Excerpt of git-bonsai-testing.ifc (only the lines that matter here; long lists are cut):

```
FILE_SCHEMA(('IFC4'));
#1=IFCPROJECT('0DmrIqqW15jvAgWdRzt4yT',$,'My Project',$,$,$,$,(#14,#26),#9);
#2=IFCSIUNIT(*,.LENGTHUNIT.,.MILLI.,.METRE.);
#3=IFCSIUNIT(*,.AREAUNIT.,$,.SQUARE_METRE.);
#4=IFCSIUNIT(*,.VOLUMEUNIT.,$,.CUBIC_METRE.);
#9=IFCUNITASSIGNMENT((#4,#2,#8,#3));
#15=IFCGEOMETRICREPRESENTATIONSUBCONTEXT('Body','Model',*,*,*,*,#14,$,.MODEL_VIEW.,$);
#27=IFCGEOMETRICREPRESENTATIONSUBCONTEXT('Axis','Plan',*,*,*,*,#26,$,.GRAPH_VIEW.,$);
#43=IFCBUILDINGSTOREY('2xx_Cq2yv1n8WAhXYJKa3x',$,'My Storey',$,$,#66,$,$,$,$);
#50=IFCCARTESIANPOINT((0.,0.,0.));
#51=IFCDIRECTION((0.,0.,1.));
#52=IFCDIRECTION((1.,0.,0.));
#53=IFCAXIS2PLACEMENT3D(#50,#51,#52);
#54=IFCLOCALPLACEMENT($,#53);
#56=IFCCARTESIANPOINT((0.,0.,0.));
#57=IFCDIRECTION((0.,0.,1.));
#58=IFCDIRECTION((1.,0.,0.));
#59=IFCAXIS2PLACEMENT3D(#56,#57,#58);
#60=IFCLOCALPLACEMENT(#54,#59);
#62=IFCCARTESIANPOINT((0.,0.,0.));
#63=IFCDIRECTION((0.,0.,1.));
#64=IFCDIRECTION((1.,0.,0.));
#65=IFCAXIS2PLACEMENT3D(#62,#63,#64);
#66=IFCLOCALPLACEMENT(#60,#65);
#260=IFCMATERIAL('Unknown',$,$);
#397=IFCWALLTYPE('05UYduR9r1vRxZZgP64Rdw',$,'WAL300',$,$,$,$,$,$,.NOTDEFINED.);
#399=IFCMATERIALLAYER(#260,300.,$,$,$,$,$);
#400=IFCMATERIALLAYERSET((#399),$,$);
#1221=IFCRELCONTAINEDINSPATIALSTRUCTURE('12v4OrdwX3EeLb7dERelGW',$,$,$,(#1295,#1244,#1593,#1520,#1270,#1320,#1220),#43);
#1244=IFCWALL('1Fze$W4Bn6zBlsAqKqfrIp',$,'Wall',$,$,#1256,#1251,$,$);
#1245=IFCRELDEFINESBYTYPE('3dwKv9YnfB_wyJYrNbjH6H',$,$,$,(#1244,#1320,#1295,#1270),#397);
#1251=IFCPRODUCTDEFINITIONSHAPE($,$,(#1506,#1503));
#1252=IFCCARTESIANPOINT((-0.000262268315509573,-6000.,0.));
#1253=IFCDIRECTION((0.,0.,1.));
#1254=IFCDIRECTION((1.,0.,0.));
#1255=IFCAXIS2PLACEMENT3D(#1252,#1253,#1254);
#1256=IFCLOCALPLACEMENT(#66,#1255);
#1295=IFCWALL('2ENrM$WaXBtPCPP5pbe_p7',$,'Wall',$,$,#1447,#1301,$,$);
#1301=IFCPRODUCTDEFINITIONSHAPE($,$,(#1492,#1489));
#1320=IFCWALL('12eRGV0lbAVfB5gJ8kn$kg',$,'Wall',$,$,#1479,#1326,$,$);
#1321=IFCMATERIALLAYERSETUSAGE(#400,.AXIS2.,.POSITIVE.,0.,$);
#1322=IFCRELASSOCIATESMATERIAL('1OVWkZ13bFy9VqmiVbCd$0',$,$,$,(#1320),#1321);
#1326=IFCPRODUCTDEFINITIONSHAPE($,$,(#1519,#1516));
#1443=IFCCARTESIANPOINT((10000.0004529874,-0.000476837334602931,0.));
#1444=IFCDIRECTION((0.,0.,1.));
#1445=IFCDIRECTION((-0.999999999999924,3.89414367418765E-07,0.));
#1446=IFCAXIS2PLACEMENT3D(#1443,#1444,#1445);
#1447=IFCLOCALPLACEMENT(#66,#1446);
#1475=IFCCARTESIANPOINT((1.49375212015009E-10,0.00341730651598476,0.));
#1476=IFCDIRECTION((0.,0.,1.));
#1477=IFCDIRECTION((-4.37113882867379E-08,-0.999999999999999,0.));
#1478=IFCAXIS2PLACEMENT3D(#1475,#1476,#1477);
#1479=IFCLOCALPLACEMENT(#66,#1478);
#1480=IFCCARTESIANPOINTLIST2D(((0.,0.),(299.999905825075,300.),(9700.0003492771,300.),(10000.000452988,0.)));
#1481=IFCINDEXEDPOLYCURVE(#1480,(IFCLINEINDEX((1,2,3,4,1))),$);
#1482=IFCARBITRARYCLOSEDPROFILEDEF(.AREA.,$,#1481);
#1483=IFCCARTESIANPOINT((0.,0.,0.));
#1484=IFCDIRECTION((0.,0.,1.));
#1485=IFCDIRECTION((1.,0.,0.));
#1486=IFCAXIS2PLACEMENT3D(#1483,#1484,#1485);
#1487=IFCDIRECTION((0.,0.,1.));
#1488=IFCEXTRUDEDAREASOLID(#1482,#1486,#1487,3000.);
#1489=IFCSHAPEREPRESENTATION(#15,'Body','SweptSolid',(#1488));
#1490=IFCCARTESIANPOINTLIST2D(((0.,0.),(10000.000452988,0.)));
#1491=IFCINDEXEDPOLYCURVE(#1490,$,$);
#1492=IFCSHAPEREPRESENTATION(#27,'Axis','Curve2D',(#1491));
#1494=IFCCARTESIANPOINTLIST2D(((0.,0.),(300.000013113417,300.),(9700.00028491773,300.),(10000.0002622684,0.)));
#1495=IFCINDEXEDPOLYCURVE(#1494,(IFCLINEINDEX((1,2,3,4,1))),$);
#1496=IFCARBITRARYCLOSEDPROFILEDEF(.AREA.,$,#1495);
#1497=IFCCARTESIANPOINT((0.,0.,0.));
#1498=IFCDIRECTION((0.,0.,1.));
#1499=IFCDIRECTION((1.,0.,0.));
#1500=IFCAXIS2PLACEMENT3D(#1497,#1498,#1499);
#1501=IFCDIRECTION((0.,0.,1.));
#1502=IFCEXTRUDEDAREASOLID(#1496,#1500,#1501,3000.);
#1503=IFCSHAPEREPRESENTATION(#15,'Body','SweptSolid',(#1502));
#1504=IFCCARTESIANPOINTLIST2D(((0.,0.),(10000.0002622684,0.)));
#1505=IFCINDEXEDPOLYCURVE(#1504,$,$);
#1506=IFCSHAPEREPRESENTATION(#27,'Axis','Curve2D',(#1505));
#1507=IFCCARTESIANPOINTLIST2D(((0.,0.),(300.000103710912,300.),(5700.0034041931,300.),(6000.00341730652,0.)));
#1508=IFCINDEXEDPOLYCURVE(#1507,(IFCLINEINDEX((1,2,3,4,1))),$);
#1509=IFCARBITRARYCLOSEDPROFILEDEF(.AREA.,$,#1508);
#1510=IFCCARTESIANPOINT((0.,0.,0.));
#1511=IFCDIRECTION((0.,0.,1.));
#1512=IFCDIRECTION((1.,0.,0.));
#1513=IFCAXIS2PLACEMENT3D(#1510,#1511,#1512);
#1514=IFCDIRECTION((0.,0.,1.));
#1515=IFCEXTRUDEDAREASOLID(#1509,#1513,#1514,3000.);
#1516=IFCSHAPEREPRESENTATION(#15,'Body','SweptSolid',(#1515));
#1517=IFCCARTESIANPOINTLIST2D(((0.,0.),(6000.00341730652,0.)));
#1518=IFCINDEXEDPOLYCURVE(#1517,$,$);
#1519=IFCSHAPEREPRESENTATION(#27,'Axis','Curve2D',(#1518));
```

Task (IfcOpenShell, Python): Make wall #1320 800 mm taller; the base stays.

```python
import ifcopenshell
import ifcopenshell.geom
import ifcopenshell.util.representation
import ifcopenshell.util.shape
import ifcopenshell.util.unit

model = ifcopenshell.open("git-bonsai-testing.ifc")
unit_scale = ifcopenshell.util.unit.calculate_unit_scale(model)
settings = ifcopenshell.geom.settings()


def volume(element):
    """Net volume in cubic metres, openings subtracted."""
    shape = ifcopenshell.geom.create_shape(settings, element)
    return ifcopenshell.util.shape.get_volume(shape.geometry)


wall = model.by_guid("12eRGV0lbAVfB5gJ8kn$kg")
before = volume(wall)

body = ifcopenshell.util.representation.get_representation(wall, "Model", "Body")
solid = body.Items[0]
old_height = solid.Depth
solid.Depth += 0.8 / unit_scale
after = volume(wall)

print(f"height {old_height:g} -> {solid.Depth:g}, volume {before:.3f} -> {after:.3f} m3")

model.write("git-bonsai-testing_edited.ifc")
```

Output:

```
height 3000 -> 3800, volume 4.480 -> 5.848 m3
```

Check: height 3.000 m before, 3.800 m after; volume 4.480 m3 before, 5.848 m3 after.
